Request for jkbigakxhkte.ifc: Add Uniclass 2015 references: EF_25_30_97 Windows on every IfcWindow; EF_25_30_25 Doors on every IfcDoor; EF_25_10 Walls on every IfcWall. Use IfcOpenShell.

First a look at what the model holds.

```python
import ifcopenshell

model = ifcopenshell.open("jkbigakxhkte.ifc")
print(model.schema)
print("classifications:", [c.Name for c in model.by_type("IfcClassification")])
for ifc_class in ("IfcDoor", "IfcRoof", "IfcStair", "IfcWall", "IfcWindow"):
    print(ifc_class, len(model.by_type(ifc_class)))
```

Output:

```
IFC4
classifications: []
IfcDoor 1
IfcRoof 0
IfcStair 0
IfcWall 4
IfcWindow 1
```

```python
import ifcopenshell
import ifcopenshell.api.classification

model = ifcopenshell.open("jkbigakxhkte.ifc")

system = ifcopenshell.api.classification.add_classification(model, classification="Uniclass 2015")

codes = {
    "IfcWindow": ("EF_25_30_97", "Windows"),
    "IfcDoor": ("EF_25_30_25", "Doors"),
    "IfcWall": ("EF_25_10", "Walls"),
}
for ifc_class, (code, name) in codes.items():
    products = model.by_type(ifc_class)
    ifcopenshell.api.classification.add_reference(
        model, products=products, classification=system, identification=code, name=name
    )
    print(code, len(products))

model.write("jkbigakxhkte_edited.ifc")
```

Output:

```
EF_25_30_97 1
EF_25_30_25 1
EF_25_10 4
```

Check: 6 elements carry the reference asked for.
